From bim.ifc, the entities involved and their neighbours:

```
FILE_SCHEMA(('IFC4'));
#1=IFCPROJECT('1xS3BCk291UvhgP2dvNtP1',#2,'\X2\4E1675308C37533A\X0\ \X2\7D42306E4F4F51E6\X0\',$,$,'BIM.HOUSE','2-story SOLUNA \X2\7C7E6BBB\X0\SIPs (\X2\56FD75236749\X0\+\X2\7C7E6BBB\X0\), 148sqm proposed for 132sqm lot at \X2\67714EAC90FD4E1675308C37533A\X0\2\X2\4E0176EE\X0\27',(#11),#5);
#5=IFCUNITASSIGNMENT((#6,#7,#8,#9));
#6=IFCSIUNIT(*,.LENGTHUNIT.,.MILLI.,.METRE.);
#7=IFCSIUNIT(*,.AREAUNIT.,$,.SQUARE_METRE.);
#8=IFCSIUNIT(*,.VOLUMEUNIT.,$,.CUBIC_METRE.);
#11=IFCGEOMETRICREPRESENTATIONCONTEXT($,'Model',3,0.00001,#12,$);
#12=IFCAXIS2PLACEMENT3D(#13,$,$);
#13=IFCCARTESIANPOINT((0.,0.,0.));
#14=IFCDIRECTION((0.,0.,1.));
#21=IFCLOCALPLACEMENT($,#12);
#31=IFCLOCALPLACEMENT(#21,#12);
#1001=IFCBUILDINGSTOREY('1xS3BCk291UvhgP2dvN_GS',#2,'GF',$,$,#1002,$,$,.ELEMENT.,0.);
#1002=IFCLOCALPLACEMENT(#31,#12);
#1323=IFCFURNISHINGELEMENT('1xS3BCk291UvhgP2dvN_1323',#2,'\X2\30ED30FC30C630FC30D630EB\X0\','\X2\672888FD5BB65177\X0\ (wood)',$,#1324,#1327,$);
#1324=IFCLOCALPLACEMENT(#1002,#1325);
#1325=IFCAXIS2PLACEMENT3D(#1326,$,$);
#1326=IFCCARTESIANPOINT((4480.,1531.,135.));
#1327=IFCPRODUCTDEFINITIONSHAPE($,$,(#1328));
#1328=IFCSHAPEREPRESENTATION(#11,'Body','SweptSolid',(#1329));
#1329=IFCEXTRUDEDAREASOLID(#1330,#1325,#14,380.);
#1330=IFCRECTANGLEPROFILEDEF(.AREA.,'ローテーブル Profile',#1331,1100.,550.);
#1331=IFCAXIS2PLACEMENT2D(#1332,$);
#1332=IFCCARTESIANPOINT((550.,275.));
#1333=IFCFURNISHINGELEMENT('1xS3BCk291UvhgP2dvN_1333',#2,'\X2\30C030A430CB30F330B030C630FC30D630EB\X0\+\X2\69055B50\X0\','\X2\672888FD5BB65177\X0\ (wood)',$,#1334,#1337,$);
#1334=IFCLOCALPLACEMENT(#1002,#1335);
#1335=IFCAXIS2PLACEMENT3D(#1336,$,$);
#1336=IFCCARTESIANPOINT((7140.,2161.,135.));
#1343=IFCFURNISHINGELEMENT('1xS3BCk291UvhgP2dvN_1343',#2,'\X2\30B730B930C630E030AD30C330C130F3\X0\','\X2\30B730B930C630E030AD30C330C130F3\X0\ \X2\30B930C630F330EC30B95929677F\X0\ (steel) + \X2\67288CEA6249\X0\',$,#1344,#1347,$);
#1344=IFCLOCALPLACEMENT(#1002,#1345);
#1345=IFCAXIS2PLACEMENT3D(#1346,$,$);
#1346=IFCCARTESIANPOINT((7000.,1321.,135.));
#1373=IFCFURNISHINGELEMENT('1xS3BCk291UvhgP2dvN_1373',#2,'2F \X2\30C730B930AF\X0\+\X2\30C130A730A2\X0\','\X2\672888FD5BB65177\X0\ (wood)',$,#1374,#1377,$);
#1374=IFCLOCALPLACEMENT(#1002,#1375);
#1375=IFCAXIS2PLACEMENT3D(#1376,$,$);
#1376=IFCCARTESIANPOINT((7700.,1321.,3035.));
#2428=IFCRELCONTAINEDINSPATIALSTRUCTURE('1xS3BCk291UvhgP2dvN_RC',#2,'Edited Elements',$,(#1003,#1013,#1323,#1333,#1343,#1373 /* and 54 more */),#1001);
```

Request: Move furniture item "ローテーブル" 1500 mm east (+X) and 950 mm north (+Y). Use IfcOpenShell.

```python
import ifcopenshell
import ifcopenshell.api.geometry
import ifcopenshell.util.placement

model = ifcopenshell.open("bim.ifc")

item = model.by_guid("1xS3BCk291UvhgP2dvN_1323")
matrix = ifcopenshell.util.placement.get_local_placement(item.ObjectPlacement)
matrix[0, 3] += 1500.0
matrix[1, 3] += 950.0
ifcopenshell.api.geometry.edit_object_placement(model, product=item, matrix=matrix, is_si=False)

print(ifcopenshell.util.placement.get_local_placement(item.ObjectPlacement).round(3) + 0.0)

model.write("bim_v2.ifc")
```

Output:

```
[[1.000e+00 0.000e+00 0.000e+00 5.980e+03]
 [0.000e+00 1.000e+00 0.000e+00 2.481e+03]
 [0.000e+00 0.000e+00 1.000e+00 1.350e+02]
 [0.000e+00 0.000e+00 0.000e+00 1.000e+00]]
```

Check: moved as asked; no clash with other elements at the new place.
